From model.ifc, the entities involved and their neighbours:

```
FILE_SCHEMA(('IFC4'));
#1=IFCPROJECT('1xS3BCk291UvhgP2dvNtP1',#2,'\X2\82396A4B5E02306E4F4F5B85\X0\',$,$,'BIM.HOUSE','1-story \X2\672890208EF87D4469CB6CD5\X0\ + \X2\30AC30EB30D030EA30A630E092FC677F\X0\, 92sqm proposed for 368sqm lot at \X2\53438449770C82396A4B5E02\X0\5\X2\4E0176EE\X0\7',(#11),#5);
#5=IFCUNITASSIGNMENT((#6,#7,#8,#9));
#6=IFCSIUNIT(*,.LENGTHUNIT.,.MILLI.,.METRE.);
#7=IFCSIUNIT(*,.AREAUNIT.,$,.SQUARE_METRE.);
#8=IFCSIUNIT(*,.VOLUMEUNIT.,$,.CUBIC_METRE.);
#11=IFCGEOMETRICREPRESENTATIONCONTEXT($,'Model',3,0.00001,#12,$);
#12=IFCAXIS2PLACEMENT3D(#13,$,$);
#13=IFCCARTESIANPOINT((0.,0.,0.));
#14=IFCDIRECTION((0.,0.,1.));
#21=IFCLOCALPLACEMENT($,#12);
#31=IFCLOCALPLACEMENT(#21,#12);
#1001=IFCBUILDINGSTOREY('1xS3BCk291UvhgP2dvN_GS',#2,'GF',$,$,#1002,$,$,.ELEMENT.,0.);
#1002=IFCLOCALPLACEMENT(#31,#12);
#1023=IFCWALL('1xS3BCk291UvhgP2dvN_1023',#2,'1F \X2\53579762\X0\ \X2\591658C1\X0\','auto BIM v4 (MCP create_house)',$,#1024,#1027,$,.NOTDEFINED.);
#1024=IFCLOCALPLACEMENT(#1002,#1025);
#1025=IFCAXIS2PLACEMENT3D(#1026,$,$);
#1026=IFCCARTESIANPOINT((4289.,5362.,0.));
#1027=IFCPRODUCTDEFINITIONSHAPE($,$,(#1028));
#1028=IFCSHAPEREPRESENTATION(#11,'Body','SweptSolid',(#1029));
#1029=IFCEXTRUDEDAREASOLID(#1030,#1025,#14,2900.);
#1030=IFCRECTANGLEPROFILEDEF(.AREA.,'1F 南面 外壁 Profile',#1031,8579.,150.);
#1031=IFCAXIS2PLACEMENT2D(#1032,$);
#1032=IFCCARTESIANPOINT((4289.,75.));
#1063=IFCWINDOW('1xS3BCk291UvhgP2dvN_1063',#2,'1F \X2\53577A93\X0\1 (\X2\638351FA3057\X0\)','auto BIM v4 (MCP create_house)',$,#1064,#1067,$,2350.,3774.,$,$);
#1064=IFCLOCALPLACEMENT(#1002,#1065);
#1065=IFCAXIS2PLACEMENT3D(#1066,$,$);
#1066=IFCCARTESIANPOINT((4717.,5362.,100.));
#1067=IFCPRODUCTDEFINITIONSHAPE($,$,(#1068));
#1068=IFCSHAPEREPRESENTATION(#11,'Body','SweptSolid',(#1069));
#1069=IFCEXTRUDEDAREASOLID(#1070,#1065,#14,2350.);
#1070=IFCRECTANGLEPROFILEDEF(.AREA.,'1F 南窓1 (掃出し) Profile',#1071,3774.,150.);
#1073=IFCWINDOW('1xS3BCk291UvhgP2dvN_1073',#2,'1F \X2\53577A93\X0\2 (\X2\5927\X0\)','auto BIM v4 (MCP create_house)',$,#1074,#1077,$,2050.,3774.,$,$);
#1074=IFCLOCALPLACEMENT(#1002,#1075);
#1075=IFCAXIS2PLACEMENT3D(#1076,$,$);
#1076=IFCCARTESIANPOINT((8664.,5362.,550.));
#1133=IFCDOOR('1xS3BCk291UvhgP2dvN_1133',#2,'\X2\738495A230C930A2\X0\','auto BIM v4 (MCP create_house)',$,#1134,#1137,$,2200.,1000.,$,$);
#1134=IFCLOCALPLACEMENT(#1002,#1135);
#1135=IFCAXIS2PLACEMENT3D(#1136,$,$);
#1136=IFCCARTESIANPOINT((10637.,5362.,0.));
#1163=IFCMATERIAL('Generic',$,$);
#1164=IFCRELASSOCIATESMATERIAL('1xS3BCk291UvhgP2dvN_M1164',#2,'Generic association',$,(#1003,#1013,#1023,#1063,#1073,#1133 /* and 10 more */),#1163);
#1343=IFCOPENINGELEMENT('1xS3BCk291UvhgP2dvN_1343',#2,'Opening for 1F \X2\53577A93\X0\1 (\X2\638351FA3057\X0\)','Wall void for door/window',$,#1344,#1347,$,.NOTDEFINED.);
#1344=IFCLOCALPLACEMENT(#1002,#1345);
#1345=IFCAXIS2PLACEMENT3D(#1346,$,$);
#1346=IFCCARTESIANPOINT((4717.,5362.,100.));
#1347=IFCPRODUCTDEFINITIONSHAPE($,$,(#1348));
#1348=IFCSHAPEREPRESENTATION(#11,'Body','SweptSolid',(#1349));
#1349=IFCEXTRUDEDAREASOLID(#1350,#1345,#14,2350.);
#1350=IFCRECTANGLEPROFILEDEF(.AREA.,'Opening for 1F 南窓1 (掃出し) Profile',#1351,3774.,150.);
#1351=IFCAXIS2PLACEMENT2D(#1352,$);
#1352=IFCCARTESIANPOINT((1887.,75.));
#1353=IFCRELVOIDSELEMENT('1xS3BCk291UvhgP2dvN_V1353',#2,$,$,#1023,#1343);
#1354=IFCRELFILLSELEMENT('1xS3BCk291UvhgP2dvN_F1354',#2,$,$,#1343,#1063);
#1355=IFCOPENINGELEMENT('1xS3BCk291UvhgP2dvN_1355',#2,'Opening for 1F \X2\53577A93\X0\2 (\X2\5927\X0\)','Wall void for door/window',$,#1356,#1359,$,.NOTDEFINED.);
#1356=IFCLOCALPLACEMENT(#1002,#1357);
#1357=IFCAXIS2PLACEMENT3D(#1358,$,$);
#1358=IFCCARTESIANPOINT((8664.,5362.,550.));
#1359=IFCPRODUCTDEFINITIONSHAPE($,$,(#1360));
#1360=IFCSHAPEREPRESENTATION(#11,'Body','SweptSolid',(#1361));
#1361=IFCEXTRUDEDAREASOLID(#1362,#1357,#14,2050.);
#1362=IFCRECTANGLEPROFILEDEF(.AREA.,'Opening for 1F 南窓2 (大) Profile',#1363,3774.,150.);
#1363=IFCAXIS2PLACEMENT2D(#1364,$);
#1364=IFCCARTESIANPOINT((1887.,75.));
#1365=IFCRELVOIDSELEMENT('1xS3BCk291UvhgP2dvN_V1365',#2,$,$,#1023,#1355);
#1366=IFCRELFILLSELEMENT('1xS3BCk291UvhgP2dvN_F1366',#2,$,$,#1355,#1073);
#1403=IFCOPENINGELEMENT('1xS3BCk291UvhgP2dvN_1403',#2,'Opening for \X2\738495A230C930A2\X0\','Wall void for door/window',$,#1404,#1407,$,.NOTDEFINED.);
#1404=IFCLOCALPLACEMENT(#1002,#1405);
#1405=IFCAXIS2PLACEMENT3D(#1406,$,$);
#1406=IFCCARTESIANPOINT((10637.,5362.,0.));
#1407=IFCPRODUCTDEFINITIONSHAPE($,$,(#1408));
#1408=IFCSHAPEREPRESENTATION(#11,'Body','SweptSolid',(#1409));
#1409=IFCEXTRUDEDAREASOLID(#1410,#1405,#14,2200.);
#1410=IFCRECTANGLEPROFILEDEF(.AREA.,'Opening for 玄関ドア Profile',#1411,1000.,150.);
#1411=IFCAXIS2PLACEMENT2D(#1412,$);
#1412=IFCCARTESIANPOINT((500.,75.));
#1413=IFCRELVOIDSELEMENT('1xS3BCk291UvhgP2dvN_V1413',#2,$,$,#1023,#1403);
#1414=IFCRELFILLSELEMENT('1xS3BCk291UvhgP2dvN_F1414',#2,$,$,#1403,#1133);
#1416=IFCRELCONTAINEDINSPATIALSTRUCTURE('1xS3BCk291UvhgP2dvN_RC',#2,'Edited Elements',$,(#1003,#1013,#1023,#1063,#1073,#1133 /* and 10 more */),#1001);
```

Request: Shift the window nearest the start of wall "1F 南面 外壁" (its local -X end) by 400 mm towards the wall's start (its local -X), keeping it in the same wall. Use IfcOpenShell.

```python
import ifcopenshell
import ifcopenshell.api.geometry
import ifcopenshell.util.placement
import ifcopenshell.util.unit

model = ifcopenshell.open("model.ifc")
unit_scale = ifcopenshell.util.unit.calculate_unit_scale(model)

window = model.by_id(1063)
opening = window.FillsVoids[0].RelatingOpeningElement
wall = opening.VoidsElements[0].RelatingBuildingElement

wall_matrix = ifcopenshell.util.placement.get_local_placement(wall.ObjectPlacement)
shift = wall_matrix[:3, 0] * -0.4 / unit_scale
before = ifcopenshell.util.placement.get_local_placement(window.ObjectPlacement)[:3, 3].copy()

# The window is not placed relative to its opening, so move both.
for product in (opening, window):
    matrix = ifcopenshell.util.placement.get_local_placement(product.ObjectPlacement)
    matrix[:3, 3] += shift
    ifcopenshell.api.geometry.edit_object_placement(model, product=product, matrix=matrix, is_si=False)

after = ifcopenshell.util.placement.get_local_placement(window.ObjectPlacement)[:3, 3]
print("window moved by", (after - before).round(3) + 0.0)

model.write("model-out.ifc")
```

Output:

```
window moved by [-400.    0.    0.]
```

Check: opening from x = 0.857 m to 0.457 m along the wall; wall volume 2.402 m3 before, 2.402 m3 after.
